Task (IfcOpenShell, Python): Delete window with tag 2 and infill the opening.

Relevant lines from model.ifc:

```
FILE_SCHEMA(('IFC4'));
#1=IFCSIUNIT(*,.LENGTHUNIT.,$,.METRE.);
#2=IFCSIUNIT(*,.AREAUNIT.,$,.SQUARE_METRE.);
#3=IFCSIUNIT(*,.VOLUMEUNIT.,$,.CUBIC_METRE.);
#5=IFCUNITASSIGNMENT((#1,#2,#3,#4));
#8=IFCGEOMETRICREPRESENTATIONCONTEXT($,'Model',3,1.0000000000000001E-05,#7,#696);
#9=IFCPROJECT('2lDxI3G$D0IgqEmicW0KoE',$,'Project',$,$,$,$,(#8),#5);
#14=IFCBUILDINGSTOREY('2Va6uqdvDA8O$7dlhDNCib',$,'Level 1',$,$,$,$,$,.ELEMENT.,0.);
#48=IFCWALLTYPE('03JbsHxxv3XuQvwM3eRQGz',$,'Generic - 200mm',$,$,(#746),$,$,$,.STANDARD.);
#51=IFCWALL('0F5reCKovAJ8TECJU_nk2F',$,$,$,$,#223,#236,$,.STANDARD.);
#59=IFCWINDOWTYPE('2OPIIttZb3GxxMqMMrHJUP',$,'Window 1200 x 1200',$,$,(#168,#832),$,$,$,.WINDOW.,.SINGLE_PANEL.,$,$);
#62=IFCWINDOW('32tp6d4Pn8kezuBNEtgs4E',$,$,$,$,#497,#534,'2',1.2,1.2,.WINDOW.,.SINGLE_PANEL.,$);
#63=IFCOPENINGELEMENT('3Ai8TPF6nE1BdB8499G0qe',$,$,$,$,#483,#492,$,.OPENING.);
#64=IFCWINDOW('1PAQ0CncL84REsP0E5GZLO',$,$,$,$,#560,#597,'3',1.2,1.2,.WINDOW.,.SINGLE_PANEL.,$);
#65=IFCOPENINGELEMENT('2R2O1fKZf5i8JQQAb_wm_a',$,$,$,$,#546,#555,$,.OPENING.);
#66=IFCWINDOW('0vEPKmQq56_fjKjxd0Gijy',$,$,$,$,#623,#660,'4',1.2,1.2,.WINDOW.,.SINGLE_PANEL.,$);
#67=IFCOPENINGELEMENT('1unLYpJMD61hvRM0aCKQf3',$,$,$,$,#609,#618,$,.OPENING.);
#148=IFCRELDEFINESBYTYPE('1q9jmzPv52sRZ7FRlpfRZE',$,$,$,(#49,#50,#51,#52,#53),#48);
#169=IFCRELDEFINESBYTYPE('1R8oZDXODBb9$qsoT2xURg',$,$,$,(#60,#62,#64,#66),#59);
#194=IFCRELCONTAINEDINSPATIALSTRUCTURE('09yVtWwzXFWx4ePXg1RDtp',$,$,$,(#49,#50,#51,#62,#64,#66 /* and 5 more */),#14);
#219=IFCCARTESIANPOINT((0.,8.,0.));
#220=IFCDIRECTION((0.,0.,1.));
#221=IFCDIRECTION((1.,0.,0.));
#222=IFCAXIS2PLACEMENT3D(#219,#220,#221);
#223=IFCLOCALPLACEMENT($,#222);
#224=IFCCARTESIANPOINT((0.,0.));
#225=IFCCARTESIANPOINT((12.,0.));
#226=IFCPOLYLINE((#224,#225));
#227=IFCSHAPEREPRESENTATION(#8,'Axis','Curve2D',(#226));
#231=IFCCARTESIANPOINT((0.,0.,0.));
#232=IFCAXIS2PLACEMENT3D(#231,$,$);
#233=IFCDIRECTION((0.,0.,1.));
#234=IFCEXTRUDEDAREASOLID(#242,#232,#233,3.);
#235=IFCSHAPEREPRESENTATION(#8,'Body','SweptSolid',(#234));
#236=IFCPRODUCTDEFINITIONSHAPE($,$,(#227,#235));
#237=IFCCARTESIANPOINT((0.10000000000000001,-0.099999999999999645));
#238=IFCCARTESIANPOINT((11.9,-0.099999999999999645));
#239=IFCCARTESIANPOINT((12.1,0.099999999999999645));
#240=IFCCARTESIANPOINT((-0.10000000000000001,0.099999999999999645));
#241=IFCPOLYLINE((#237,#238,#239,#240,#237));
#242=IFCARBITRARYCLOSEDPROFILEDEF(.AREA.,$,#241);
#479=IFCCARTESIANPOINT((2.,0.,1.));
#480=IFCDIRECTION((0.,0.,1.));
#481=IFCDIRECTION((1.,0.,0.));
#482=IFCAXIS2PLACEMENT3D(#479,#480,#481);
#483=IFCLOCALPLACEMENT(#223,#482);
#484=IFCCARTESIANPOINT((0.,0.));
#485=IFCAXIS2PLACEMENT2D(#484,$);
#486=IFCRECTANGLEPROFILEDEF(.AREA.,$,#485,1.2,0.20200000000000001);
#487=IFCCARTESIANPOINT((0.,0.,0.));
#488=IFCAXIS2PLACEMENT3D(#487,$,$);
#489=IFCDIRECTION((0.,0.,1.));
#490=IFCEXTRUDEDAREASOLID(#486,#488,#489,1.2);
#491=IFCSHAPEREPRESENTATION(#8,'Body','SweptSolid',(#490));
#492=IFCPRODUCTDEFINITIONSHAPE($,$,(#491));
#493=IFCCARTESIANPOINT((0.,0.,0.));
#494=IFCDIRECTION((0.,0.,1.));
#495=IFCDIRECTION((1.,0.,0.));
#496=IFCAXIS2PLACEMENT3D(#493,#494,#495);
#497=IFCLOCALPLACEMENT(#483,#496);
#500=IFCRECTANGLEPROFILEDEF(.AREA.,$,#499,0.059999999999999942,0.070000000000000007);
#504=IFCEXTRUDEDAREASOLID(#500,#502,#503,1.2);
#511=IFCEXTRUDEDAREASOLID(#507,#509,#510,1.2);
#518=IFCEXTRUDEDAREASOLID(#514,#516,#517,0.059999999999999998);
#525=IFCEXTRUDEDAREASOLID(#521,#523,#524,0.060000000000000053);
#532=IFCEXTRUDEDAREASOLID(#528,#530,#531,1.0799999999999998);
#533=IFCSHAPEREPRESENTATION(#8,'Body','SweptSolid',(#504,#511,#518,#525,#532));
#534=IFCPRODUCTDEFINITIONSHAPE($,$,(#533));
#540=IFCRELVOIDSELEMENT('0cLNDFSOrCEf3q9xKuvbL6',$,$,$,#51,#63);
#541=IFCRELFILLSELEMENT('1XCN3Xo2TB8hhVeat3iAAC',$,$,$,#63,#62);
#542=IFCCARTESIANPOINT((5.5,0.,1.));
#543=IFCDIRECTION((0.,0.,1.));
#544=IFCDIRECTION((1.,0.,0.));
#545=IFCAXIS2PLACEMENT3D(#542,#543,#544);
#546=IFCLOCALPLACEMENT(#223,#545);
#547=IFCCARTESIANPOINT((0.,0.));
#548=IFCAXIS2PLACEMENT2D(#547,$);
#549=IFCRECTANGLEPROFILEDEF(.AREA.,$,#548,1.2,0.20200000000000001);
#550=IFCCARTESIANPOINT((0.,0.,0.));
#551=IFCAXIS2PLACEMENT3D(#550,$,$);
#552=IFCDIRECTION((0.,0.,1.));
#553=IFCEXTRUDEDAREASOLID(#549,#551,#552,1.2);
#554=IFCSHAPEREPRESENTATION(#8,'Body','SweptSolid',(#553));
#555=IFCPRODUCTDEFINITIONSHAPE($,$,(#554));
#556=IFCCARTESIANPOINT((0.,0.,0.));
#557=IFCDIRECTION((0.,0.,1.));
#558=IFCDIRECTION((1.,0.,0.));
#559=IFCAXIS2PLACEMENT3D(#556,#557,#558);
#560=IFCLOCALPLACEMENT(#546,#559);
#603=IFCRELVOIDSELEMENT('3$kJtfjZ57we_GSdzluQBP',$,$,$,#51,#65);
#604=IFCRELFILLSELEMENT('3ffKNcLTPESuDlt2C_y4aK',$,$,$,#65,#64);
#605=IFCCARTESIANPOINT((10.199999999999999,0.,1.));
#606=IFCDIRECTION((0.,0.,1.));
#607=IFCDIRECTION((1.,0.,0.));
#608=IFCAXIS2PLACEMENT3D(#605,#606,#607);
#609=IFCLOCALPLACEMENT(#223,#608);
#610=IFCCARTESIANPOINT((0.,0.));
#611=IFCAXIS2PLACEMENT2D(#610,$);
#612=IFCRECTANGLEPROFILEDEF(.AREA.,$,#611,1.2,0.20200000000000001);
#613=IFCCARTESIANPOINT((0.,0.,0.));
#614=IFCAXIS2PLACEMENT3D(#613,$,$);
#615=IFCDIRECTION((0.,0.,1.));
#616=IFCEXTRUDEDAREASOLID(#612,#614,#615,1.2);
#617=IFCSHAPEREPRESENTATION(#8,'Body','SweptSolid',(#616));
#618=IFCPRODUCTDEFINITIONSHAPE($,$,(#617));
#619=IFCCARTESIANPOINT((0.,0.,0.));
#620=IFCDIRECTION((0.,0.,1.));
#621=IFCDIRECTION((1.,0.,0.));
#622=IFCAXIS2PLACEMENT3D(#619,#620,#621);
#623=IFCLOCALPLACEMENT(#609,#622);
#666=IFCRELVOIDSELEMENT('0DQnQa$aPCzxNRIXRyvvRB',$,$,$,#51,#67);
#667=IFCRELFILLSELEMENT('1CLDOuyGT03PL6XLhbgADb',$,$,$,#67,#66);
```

```python
import ifcopenshell
import ifcopenshell.api.feature
import ifcopenshell.api.root
import ifcopenshell.geom
import ifcopenshell.util.shape

model = ifcopenshell.open("model.ifc")
settings = ifcopenshell.geom.settings()


def volume(element):
    """Net volume in cubic metres, openings subtracted."""
    shape = ifcopenshell.geom.create_shape(settings, element)
    return ifcopenshell.util.shape.get_volume(shape.geometry)


window = model.by_id(62)
opening = window.FillsVoids[0].RelatingOpeningElement
wall = opening.VoidsElements[0].RelatingBuildingElement
before = volume(wall)

ifcopenshell.api.root.remove_product(model, product=window)
ifcopenshell.api.feature.remove_feature(model, feature=opening)

after = volume(wall)

print(f"wall volume {before:.3f} -> {after:.3f} m3")

model.write("model_v2.ifc")
```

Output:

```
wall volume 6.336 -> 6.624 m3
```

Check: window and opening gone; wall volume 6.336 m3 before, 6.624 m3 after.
